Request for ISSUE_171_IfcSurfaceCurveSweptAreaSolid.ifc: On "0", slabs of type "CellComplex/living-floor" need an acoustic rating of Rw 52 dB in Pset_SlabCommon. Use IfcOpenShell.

First a look at what the model holds.

```python
import ifcopenshell
import ifcopenshell.util.element

model = ifcopenshell.open("ISSUE_171_IfcSurfaceCurveSweptAreaSolid.ifc")
print(model.schema)
storey = next(s for s in model.by_type("IfcBuildingStorey") if s.Name == "0")
slabs = [e for e in ifcopenshell.util.element.get_decomposition(storey) if e.is_a("IfcSlab")]
seen = {}
for e in slabs:
    element_type = ifcopenshell.util.element.get_type(e)
    key = (element_type.Name if element_type != e and element_type else None, ifcopenshell.util.element.get_pset(e, "Pset_SlabCommon", "AcousticRating"))
    seen[key] = seen.get(key, 0) + 1
for (name, value), count in sorted(seen.items(), key=str):
    print(count, "x", name, "|", value)
```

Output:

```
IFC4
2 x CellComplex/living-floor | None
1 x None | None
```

```python
import ifcopenshell
import ifcopenshell.api.pset
import ifcopenshell.util.element

model = ifcopenshell.open("ISSUE_171_IfcSurfaceCurveSweptAreaSolid.ifc")

storey = next(s for s in model.by_type("IfcBuildingStorey") if s.Name == "0")
slabs = [e for e in ifcopenshell.util.element.get_decomposition(storey) if e.is_a("IfcSlab")]

count = 0
for e in slabs:
    element_type = ifcopenshell.util.element.get_type(e)
    if element_type in (None, e) or element_type.Name != "CellComplex/living-floor":
        continue
    # add_pset returns the element's existing set when there is one.
    pset = ifcopenshell.api.pset.add_pset(model, product=e, name="Pset_SlabCommon")
    ifcopenshell.api.pset.edit_pset(model, pset=pset, properties={"AcousticRating": "Rw 52 dB"})
    count += 1

print(count, "slabs updated")

model.write("ISSUE_171_IfcSurfaceCurveSweptAreaSolid_updated.ifc")
```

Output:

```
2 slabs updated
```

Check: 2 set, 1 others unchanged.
